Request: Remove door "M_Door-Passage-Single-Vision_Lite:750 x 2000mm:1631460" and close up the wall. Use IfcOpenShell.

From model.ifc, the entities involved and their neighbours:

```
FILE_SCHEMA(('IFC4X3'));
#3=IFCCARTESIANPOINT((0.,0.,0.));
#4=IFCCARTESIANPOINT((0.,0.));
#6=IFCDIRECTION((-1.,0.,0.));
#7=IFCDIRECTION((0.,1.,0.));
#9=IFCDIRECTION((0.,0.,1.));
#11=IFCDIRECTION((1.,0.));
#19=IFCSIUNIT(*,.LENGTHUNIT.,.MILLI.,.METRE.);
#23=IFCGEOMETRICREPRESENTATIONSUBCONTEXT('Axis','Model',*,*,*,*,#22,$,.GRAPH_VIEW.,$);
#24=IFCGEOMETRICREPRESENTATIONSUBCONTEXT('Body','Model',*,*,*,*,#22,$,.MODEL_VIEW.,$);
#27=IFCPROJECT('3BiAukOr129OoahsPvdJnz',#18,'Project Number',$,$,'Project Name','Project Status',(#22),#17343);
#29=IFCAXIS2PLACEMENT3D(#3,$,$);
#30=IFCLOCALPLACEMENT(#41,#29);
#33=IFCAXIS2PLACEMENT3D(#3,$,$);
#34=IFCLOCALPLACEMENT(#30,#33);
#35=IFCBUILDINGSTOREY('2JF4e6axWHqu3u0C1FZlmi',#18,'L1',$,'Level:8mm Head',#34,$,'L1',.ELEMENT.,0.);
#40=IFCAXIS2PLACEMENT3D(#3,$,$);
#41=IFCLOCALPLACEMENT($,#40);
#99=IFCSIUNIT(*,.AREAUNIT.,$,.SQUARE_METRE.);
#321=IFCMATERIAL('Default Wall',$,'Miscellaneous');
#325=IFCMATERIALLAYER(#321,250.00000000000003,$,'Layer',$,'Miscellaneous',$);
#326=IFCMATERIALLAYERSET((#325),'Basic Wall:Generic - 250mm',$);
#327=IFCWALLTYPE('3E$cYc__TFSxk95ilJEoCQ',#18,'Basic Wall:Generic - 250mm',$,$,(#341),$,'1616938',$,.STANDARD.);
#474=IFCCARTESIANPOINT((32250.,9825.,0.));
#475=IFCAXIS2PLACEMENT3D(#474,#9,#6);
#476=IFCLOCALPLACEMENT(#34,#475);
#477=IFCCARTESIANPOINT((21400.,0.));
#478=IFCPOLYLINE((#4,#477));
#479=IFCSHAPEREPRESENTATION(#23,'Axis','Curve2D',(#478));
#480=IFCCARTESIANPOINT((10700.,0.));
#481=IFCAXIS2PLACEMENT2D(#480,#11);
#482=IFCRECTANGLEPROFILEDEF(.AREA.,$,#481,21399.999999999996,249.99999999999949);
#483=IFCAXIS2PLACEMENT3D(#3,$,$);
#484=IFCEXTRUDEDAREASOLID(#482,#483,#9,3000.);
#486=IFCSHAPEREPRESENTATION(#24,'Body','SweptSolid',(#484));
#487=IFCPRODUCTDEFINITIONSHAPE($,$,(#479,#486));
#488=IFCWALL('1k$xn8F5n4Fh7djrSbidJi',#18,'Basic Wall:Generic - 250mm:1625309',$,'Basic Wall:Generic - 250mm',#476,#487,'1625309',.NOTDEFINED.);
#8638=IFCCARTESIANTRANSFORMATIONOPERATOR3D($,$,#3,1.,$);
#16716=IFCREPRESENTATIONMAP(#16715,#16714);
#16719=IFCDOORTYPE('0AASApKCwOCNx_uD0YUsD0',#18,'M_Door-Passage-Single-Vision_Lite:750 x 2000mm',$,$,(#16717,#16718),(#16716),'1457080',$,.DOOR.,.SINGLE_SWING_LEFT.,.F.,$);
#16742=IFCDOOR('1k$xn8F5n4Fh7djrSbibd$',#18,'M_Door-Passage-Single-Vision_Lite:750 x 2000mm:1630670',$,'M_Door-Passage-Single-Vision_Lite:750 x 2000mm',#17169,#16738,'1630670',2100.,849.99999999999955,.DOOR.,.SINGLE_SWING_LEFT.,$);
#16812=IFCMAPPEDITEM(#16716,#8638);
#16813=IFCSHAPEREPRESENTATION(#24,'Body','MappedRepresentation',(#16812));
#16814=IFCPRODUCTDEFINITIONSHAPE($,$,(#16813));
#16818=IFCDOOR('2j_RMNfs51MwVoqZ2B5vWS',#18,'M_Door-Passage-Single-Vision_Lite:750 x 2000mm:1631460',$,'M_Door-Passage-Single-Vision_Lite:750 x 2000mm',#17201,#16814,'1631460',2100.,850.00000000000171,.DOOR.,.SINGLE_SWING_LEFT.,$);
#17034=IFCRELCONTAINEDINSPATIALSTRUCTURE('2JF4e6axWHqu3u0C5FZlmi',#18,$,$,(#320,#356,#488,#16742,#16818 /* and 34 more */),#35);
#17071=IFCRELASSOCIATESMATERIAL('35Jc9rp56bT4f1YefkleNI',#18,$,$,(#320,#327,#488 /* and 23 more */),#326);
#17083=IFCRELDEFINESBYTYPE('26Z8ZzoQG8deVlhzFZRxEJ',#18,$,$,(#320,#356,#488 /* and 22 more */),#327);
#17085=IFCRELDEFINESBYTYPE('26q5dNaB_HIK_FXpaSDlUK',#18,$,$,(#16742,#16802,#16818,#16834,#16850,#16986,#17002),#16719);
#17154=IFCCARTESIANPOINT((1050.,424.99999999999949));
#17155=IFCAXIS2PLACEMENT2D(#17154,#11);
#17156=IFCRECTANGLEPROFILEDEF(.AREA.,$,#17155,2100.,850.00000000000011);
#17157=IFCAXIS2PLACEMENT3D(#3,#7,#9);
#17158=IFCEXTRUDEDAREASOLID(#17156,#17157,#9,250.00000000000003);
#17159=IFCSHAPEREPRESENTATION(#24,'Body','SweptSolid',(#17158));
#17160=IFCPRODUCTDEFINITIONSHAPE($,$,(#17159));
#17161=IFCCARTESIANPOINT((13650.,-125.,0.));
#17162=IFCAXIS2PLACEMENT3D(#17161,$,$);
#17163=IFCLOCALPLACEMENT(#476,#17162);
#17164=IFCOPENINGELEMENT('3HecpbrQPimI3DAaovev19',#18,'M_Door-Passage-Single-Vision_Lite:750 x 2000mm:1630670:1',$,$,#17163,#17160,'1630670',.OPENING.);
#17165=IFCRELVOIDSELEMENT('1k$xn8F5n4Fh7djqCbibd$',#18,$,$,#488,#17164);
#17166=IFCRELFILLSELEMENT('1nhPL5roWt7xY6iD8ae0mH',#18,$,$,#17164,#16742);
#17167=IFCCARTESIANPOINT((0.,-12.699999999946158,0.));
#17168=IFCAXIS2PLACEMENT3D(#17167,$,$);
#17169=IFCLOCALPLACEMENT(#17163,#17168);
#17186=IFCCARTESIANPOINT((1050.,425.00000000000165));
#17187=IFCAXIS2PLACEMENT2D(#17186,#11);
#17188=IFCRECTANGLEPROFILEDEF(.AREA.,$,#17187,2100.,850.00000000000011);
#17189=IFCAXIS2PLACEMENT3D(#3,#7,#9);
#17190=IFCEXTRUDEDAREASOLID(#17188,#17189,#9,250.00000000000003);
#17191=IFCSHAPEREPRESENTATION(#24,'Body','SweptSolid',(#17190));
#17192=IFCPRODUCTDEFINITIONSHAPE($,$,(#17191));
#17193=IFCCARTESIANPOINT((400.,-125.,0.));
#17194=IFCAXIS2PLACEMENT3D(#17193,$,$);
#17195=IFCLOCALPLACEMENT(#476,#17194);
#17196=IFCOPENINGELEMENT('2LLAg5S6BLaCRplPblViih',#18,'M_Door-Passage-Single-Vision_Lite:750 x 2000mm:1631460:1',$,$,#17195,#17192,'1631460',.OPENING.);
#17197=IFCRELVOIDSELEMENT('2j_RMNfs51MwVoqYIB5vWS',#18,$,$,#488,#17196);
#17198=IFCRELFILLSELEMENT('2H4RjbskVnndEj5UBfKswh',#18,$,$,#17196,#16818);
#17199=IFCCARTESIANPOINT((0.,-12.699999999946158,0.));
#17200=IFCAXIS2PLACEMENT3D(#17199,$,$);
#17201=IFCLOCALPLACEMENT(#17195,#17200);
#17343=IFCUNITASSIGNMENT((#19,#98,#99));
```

```python
import ifcopenshell
import ifcopenshell.api.feature
import ifcopenshell.api.root
import ifcopenshell.geom
import ifcopenshell.util.shape

model = ifcopenshell.open("model.ifc")
settings = ifcopenshell.geom.settings()


def volume(element):
    """Net volume in cubic metres, openings subtracted."""
    shape = ifcopenshell.geom.create_shape(settings, element)
    return ifcopenshell.util.shape.get_volume(shape.geometry)


door = model.by_guid("2j_RMNfs51MwVoqZ2B5vWS")
opening = door.FillsVoids[0].RelatingOpeningElement
wall = opening.VoidsElements[0].RelatingBuildingElement
before = volume(wall)

ifcopenshell.api.root.remove_product(model, product=door)
ifcopenshell.api.feature.remove_feature(model, feature=opening)

after = volume(wall)

print(f"wall volume {before:.3f} -> {after:.3f} m3")

model.write("model-out.ifc")
```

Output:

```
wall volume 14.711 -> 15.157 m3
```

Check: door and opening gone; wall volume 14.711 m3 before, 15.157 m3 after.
